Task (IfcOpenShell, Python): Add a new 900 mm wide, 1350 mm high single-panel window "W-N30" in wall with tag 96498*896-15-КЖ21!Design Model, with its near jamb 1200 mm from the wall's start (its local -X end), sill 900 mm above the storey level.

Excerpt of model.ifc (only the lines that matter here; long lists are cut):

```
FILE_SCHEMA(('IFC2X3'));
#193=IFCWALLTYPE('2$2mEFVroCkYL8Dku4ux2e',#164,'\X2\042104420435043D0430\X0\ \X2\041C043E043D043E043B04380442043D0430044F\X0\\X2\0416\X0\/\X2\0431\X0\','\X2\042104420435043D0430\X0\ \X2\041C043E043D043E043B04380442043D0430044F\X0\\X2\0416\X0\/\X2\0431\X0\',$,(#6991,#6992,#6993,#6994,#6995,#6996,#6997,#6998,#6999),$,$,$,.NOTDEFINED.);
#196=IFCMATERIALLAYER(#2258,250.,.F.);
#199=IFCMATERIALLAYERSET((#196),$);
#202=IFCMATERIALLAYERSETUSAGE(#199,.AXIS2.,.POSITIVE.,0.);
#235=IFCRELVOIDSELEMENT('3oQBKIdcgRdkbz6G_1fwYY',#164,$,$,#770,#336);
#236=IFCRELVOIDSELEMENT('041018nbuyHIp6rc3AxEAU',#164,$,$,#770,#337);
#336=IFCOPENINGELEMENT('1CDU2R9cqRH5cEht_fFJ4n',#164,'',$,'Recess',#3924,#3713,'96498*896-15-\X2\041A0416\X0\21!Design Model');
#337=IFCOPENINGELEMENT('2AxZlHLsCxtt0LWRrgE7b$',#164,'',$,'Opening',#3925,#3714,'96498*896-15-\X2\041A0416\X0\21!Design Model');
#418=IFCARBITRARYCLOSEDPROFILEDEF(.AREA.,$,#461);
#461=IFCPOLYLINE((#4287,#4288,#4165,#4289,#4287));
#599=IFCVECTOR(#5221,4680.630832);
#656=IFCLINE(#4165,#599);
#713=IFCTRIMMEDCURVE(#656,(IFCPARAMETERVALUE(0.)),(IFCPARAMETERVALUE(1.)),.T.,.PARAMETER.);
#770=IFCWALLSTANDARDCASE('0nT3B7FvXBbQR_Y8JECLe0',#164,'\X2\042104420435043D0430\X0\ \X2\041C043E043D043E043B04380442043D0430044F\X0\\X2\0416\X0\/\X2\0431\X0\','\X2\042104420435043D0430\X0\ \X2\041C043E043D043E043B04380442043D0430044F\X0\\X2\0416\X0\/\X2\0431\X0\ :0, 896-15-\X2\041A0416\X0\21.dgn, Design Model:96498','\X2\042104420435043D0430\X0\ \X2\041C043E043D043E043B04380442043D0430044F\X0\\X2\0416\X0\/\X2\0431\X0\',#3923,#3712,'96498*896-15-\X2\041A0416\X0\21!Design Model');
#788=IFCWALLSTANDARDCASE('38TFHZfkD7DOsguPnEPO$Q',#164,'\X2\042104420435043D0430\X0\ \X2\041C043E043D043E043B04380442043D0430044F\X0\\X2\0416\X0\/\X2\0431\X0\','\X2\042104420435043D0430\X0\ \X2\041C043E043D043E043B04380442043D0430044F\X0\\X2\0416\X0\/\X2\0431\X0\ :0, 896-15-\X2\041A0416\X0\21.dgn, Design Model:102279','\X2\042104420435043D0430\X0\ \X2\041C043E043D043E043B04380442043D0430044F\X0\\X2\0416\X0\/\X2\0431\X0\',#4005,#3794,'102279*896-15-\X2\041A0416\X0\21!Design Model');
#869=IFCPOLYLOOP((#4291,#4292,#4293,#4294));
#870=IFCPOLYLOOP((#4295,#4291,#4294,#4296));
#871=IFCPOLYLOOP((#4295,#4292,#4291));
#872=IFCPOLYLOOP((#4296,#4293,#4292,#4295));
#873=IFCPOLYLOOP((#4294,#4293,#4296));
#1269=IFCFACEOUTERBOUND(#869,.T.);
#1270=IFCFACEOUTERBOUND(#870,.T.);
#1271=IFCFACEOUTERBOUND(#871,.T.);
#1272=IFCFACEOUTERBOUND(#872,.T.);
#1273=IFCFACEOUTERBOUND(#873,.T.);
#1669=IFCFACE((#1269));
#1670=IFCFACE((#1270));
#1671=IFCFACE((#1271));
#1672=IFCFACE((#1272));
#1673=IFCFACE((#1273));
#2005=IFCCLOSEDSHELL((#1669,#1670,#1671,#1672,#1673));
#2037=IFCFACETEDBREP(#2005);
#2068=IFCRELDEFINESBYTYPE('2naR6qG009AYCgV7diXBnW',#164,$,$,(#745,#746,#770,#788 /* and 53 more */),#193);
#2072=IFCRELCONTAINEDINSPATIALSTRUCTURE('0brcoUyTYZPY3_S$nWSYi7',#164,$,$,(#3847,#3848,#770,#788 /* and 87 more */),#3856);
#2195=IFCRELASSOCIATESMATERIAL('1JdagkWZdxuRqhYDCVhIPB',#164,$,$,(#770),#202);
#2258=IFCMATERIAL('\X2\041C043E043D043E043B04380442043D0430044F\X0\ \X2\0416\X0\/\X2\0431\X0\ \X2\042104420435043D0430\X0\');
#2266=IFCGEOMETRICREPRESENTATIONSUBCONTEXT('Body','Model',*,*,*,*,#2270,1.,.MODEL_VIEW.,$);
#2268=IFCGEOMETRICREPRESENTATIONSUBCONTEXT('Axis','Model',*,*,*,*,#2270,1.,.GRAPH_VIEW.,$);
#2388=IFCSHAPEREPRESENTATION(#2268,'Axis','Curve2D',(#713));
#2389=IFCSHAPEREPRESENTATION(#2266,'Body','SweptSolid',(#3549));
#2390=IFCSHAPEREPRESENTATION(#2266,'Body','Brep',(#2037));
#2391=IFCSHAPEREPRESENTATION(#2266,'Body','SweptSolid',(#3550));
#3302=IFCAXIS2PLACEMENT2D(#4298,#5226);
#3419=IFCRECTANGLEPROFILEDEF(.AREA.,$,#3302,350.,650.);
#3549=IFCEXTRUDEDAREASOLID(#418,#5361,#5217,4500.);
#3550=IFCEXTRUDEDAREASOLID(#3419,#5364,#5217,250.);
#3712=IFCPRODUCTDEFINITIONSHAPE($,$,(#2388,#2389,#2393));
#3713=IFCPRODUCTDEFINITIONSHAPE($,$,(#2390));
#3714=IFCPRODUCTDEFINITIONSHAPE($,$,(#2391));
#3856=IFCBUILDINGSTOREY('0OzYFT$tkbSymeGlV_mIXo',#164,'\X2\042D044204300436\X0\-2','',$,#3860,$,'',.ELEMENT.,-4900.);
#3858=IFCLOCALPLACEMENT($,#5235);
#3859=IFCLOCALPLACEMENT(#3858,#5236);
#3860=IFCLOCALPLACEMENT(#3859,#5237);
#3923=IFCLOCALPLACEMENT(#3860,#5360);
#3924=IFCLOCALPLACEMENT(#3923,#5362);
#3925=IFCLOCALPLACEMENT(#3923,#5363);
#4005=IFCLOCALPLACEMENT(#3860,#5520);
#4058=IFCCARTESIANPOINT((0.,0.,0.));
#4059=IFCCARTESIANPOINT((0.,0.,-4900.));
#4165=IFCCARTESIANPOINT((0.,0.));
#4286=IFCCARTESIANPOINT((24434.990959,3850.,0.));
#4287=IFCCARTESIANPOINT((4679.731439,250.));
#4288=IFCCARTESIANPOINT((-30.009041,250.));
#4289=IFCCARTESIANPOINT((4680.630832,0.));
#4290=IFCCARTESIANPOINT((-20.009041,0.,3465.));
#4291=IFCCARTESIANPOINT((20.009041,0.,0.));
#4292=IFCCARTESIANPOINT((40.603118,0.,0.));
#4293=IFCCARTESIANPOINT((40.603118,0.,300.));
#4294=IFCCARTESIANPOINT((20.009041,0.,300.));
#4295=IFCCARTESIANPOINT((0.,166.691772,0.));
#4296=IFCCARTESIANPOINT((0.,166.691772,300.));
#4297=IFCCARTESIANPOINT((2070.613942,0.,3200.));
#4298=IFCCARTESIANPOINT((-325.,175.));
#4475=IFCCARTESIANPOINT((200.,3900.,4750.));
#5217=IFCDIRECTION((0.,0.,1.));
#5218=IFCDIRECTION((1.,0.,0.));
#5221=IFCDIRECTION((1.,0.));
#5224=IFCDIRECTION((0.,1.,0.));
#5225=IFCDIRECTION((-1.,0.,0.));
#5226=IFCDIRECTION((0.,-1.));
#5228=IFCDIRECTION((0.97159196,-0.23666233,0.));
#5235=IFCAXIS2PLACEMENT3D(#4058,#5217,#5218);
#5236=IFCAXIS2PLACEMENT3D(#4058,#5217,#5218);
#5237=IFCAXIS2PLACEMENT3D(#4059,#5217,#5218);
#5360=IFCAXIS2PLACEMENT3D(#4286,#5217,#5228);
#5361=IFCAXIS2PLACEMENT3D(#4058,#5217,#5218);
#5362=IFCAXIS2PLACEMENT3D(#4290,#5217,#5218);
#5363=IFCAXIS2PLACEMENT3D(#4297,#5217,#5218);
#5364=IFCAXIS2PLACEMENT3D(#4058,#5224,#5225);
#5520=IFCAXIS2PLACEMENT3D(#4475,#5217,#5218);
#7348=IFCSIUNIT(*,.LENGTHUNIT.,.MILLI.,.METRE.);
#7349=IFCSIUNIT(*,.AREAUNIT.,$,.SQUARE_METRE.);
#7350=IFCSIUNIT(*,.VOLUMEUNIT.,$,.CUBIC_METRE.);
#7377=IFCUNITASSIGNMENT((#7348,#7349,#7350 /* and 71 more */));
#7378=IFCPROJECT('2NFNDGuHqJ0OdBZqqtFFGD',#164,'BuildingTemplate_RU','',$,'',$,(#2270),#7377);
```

```python
import numpy as np
import ifcopenshell
import ifcopenshell.api.feature
import ifcopenshell.api.geometry
import ifcopenshell.api.root
import ifcopenshell.api.spatial
import ifcopenshell.api.type
import ifcopenshell.geom
import ifcopenshell.util.element
import ifcopenshell.util.placement
import ifcopenshell.util.representation
import ifcopenshell.util.shape
import ifcopenshell.util.unit

model = ifcopenshell.open("model.ifc")
unit_scale = ifcopenshell.util.unit.calculate_unit_scale(model)
settings = ifcopenshell.geom.settings()


def volume(element):
    """Net volume in cubic metres, openings subtracted."""
    shape = ifcopenshell.geom.create_shape(settings, element)
    return ifcopenshell.util.shape.get_volume(shape.geometry)


wall = model.by_guid("0nT3B7FvXBbQR_Y8JECLe0")
storey = ifcopenshell.util.element.get_container(wall, ifc_class="IfcBuildingStorey")
context = ifcopenshell.util.representation.get_context(model, "Model", "Body", "MODEL_VIEW")
before = volume(wall)

width, height, from_end, sill = 0.9, 1.35, 1.2, 0.9  # metres

# The wall runs along its own X axis, and the end named is its -X end.
wall_shape = ifcopenshell.geom.create_shape(settings, wall)
x, y, z = ifcopenshell.util.shape.get_vertices(wall_shape.geometry).T
start = x.min() + from_end
face, thickness = float(y.min()), float(y.max() - y.min())
wall_matrix = ifcopenshell.util.placement.get_local_placement(wall.ObjectPlacement)
level = ifcopenshell.util.placement.get_local_placement(storey.ObjectPlacement)[2, 3]


def in_wall(x, y):
    """Placement at x, y metres in the wall's axes, at sill height."""
    matrix = wall_matrix.copy()
    matrix[:, 3] = wall_matrix @ np.array([x / unit_scale, y / unit_scale, 0.0, 1.0])
    matrix[2, 3] = level + sill / unit_scale
    return matrix


# Opening: a box that overshoots both wall faces by 50 mm.
opening = ifcopenshell.api.root.create_entity(model, ifc_class="IfcOpeningElement")
box = ifcopenshell.api.geometry.add_wall_representation(
    model, context=context, length=width, height=height, thickness=thickness + 0.1
)
ifcopenshell.api.geometry.assign_representation(model, product=opening, representation=box)
ifcopenshell.api.geometry.edit_object_placement(model, product=opening, matrix=in_wall(start, face - 0.05), is_si=False)
ifcopenshell.api.feature.add_feature(model, feature=opening, element=wall)

window = ifcopenshell.api.root.create_entity(model, ifc_class="IfcWindow", name="W-N30")
window.OverallWidth, window.OverallHeight = width / unit_scale, height / unit_scale
body = ifcopenshell.api.geometry.add_window_representation(
    model,
    context=context,
    overall_width=window.OverallWidth,
    overall_height=window.OverallHeight,
    partition_type="SINGLE_PANEL",
)
ifcopenshell.api.geometry.assign_representation(model, product=window, representation=body)
ifcopenshell.api.spatial.assign_container(model, products=[window], relating_structure=storey)
fills = ifcopenshell.api.feature.add_filling(model, opening=opening, element=window)
fills.OwnerHistory = window.OwnerHistory  # required in IFC2X3

# IFC2X3 keeps the operation on the window style.
style = ifcopenshell.api.root.create_entity(model, ifc_class="IfcWindowStyle", name="W-N30")
style.OperationType, style.ConstructionType = "SINGLE_PANEL", "NOTDEFINED"
style.ParameterTakesPrecedence = style.Sizeable = False
ifcopenshell.api.type.assign_type(model, related_objects=[window], relating_type=style)

# Centre the window in the wall's thickness.
ifcopenshell.api.geometry.edit_object_placement(model, product=window, matrix=in_wall(start, face), is_si=False)
window_shape = ifcopenshell.geom.create_shape(settings, window)
depth = ifcopenshell.util.shape.get_vertices(window_shape.geometry)[:, 1]
offset = face + thickness / 2 - (depth.min() + depth.max()) / 2
ifcopenshell.api.geometry.edit_object_placement(model, product=window, matrix=in_wall(start, offset), is_si=False)

after = volume(wall)

print(f"wall volume {before:.3f} -> {after:.3f} m3")

model.write("model_updated.ifc")
```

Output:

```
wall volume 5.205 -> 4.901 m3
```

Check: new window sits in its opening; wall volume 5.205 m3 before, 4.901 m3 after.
